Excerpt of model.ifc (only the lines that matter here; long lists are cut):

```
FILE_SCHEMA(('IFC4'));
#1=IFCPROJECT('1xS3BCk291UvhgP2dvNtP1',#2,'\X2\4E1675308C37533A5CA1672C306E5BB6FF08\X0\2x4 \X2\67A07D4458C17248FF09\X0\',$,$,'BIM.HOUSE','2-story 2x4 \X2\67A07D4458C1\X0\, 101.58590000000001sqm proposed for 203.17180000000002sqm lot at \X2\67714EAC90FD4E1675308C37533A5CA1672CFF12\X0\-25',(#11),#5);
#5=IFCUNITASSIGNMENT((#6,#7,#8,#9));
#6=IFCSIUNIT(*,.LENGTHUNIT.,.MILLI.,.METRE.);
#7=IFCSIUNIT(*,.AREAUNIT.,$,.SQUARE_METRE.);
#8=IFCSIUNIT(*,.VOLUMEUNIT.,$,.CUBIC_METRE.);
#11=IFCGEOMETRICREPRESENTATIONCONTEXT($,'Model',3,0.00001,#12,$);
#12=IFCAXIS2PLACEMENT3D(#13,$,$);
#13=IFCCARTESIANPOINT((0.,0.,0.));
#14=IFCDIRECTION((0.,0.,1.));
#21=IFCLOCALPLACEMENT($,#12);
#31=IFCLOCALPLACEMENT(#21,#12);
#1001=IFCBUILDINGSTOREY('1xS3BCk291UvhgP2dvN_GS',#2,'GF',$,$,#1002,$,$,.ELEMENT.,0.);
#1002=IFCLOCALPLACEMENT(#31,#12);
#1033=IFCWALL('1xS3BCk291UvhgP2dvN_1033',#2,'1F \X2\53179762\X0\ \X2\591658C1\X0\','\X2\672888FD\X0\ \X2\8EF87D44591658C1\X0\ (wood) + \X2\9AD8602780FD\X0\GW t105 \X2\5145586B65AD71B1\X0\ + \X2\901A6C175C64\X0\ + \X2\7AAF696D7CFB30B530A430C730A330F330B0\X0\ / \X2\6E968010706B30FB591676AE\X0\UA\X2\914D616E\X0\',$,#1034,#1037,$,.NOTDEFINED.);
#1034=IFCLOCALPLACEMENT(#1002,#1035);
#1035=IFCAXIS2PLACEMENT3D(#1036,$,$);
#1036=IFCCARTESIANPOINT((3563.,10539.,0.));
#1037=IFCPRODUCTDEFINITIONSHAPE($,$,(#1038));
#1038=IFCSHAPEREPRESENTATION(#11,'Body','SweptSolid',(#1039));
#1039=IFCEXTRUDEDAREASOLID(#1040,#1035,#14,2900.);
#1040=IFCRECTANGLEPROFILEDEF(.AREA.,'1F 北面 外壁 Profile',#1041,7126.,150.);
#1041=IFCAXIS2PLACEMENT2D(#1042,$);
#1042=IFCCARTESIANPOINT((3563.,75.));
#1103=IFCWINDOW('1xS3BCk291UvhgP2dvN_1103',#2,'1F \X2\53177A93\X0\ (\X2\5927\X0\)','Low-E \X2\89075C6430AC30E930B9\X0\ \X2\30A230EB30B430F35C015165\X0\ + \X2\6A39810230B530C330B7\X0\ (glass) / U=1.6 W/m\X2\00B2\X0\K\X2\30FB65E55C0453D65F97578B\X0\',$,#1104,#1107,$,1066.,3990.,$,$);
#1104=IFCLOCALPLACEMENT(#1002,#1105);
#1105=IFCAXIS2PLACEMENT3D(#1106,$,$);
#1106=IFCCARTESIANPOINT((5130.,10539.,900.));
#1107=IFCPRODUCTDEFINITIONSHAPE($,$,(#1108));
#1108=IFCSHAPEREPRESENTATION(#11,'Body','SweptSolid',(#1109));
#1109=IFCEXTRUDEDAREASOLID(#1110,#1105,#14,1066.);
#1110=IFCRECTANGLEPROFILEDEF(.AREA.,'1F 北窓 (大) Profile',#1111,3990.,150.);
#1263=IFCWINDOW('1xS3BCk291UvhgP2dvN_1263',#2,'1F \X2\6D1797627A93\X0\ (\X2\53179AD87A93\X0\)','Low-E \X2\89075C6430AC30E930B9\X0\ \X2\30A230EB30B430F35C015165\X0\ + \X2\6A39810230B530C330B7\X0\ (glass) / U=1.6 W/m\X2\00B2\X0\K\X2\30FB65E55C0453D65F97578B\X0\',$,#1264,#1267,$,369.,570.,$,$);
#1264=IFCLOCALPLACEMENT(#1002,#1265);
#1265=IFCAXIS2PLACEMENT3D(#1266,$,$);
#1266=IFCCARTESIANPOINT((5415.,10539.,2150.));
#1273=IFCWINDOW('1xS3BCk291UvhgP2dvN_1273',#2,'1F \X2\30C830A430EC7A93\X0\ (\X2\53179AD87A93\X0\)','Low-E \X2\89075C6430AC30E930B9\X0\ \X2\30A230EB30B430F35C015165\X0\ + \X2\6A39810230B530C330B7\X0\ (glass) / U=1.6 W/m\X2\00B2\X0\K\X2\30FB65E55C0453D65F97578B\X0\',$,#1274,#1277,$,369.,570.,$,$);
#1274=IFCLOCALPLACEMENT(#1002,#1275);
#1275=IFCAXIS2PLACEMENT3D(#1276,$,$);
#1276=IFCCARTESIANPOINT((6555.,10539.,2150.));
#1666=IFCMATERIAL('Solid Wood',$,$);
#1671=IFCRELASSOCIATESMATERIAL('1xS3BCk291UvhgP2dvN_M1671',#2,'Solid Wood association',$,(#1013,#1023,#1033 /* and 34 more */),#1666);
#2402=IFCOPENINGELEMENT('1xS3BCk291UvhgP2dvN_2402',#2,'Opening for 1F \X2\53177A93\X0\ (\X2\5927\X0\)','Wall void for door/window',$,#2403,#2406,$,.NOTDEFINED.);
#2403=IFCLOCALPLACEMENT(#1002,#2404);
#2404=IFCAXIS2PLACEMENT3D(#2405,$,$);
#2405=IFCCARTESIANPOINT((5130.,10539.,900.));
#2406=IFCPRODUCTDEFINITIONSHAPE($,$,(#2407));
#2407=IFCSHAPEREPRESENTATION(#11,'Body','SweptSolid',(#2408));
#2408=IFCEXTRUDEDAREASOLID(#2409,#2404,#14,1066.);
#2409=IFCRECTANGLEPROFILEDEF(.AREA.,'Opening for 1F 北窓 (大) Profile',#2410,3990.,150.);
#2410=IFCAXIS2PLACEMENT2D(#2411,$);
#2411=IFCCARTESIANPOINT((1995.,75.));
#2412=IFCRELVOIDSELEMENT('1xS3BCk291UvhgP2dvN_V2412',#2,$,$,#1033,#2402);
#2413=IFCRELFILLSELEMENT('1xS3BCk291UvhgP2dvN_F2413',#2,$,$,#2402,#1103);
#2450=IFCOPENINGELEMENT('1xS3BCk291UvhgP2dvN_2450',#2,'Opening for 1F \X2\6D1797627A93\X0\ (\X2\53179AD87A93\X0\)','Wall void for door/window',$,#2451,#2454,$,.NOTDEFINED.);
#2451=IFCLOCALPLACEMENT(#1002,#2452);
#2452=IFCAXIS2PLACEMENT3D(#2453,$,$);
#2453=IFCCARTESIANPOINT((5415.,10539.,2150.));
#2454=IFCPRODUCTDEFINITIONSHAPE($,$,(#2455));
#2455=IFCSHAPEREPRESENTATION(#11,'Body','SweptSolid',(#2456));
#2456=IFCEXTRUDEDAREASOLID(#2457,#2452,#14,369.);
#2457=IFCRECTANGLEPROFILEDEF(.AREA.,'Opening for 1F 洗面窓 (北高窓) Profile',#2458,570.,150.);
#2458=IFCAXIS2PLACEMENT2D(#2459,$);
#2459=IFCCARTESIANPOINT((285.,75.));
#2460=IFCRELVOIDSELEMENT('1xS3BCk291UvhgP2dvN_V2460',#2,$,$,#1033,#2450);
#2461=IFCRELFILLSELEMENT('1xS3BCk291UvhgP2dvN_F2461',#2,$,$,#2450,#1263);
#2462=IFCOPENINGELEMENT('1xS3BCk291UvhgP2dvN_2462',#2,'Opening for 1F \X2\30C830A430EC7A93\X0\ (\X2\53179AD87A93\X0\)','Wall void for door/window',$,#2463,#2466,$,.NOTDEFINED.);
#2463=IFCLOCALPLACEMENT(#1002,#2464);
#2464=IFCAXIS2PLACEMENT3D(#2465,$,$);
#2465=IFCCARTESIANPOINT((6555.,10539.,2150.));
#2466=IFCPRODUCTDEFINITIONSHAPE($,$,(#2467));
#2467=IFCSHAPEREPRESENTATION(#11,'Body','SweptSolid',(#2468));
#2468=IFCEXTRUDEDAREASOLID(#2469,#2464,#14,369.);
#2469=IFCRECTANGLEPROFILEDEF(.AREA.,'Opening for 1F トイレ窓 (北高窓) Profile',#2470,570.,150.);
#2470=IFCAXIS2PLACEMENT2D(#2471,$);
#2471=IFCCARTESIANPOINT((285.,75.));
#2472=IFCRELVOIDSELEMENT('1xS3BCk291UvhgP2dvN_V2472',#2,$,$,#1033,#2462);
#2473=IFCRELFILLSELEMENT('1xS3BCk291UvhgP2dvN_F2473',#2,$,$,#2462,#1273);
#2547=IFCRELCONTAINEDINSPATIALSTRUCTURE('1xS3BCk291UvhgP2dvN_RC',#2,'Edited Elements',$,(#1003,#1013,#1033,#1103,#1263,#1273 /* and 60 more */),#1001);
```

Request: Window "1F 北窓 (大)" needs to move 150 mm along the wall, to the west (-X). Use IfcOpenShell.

```python
import ifcopenshell
import ifcopenshell.api.geometry
import ifcopenshell.util.placement
import ifcopenshell.util.unit

model = ifcopenshell.open("model.ifc")
unit_scale = ifcopenshell.util.unit.calculate_unit_scale(model)

window = model.by_id(1103)
opening = window.FillsVoids[0].RelatingOpeningElement
wall = opening.VoidsElements[0].RelatingBuildingElement

wall_matrix = ifcopenshell.util.placement.get_local_placement(wall.ObjectPlacement)
shift = wall_matrix[:3, 0] * -0.15 / unit_scale
before = ifcopenshell.util.placement.get_local_placement(window.ObjectPlacement)[:3, 3].copy()

# The window is not placed relative to its opening, so move both.
for product in (opening, window):
    matrix = ifcopenshell.util.placement.get_local_placement(product.ObjectPlacement)
    matrix[:3, 3] += shift
    ifcopenshell.api.geometry.edit_object_placement(model, product=product, matrix=matrix, is_si=False)

after = ifcopenshell.util.placement.get_local_placement(window.ObjectPlacement)[:3, 3]
print("window moved by", (after - before).round(3) + 0.0)

model.write("model_updated.ifc")
```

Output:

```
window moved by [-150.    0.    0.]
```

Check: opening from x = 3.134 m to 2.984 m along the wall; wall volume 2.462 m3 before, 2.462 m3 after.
